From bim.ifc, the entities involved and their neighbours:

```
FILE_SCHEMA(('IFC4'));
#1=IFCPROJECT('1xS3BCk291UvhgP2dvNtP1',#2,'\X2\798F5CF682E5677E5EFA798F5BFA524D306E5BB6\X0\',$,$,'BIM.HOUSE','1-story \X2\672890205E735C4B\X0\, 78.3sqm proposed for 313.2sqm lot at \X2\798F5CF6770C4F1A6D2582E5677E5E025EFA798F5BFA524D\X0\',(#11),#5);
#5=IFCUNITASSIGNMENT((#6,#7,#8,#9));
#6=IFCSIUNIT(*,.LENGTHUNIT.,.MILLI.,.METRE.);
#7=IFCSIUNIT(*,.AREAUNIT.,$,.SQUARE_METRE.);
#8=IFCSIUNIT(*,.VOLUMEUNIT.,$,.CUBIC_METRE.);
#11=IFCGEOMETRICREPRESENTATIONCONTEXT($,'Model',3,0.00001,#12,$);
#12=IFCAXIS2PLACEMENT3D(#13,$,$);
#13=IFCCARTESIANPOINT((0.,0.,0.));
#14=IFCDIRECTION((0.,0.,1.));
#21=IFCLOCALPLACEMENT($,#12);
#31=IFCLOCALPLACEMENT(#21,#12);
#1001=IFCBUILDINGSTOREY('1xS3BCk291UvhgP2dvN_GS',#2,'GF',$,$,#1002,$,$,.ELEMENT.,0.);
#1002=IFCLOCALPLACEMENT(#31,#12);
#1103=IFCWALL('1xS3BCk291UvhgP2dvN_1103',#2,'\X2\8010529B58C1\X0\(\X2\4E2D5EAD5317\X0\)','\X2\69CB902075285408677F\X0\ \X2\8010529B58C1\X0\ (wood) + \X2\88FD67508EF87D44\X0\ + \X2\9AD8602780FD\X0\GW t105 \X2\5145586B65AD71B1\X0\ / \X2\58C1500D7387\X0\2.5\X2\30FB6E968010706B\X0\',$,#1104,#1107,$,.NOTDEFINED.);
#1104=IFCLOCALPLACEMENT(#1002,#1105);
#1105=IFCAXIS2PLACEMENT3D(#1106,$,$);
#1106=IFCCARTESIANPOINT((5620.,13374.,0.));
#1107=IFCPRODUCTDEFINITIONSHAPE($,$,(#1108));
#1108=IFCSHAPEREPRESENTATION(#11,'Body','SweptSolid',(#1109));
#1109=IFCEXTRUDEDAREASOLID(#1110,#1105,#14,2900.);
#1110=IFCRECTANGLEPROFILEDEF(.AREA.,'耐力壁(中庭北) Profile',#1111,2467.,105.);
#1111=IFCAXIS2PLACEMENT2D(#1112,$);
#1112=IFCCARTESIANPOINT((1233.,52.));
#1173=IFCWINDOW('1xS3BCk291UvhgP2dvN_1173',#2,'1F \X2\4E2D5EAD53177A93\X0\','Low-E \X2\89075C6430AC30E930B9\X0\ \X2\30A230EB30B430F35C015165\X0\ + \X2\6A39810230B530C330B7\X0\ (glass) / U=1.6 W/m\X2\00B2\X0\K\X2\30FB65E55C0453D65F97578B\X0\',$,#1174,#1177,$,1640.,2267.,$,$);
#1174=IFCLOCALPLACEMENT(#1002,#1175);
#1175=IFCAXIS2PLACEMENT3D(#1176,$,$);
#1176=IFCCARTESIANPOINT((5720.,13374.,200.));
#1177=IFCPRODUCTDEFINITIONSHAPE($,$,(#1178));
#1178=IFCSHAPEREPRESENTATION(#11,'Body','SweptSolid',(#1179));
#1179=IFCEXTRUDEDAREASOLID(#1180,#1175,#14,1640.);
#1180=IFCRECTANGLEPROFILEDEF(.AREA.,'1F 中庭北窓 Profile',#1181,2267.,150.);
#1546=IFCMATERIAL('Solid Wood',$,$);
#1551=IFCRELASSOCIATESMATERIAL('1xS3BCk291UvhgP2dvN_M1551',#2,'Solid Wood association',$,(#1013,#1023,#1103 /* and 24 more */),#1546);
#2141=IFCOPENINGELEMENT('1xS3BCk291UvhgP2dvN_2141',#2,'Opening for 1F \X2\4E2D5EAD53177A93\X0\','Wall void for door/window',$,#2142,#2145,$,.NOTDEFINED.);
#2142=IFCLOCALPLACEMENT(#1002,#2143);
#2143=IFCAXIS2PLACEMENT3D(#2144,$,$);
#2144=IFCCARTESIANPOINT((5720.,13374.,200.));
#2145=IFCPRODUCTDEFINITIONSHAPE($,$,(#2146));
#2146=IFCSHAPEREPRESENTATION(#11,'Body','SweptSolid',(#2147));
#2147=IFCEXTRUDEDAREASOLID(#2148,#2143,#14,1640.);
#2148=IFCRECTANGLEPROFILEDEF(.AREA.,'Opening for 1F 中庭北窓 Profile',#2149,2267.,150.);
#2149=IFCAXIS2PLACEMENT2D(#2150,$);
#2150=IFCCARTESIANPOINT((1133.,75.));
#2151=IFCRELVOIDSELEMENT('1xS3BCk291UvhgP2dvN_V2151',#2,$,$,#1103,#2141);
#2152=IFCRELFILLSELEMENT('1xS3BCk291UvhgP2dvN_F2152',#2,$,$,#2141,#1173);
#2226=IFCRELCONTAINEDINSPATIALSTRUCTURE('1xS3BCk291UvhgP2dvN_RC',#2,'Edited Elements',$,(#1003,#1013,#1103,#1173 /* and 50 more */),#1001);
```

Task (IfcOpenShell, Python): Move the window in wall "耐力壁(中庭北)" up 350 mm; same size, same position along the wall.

```python
import numpy as np
import ifcopenshell
import ifcopenshell.api.geometry
import ifcopenshell.util.placement
import ifcopenshell.util.unit

model = ifcopenshell.open("bim.ifc")
unit_scale = ifcopenshell.util.unit.calculate_unit_scale(model)

window = model.by_guid("1xS3BCk291UvhgP2dvN_1173")
opening = window.FillsVoids[0].RelatingOpeningElement
dz = 0.35 / unit_scale

shift = np.array([0.0, 0.0, dz])
# The window is not placed relative to its opening, so move both.
for product in (opening, window):
    matrix = ifcopenshell.util.placement.get_local_placement(product.ObjectPlacement)
    matrix[:3, 3] += shift
    ifcopenshell.api.geometry.edit_object_placement(model, product=product, matrix=matrix, is_si=False)

print(f"moved by {dz * unit_scale:+.3f} m")

model.write("bim_edited.ifc")
```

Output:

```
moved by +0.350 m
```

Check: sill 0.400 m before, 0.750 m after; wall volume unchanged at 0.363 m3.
